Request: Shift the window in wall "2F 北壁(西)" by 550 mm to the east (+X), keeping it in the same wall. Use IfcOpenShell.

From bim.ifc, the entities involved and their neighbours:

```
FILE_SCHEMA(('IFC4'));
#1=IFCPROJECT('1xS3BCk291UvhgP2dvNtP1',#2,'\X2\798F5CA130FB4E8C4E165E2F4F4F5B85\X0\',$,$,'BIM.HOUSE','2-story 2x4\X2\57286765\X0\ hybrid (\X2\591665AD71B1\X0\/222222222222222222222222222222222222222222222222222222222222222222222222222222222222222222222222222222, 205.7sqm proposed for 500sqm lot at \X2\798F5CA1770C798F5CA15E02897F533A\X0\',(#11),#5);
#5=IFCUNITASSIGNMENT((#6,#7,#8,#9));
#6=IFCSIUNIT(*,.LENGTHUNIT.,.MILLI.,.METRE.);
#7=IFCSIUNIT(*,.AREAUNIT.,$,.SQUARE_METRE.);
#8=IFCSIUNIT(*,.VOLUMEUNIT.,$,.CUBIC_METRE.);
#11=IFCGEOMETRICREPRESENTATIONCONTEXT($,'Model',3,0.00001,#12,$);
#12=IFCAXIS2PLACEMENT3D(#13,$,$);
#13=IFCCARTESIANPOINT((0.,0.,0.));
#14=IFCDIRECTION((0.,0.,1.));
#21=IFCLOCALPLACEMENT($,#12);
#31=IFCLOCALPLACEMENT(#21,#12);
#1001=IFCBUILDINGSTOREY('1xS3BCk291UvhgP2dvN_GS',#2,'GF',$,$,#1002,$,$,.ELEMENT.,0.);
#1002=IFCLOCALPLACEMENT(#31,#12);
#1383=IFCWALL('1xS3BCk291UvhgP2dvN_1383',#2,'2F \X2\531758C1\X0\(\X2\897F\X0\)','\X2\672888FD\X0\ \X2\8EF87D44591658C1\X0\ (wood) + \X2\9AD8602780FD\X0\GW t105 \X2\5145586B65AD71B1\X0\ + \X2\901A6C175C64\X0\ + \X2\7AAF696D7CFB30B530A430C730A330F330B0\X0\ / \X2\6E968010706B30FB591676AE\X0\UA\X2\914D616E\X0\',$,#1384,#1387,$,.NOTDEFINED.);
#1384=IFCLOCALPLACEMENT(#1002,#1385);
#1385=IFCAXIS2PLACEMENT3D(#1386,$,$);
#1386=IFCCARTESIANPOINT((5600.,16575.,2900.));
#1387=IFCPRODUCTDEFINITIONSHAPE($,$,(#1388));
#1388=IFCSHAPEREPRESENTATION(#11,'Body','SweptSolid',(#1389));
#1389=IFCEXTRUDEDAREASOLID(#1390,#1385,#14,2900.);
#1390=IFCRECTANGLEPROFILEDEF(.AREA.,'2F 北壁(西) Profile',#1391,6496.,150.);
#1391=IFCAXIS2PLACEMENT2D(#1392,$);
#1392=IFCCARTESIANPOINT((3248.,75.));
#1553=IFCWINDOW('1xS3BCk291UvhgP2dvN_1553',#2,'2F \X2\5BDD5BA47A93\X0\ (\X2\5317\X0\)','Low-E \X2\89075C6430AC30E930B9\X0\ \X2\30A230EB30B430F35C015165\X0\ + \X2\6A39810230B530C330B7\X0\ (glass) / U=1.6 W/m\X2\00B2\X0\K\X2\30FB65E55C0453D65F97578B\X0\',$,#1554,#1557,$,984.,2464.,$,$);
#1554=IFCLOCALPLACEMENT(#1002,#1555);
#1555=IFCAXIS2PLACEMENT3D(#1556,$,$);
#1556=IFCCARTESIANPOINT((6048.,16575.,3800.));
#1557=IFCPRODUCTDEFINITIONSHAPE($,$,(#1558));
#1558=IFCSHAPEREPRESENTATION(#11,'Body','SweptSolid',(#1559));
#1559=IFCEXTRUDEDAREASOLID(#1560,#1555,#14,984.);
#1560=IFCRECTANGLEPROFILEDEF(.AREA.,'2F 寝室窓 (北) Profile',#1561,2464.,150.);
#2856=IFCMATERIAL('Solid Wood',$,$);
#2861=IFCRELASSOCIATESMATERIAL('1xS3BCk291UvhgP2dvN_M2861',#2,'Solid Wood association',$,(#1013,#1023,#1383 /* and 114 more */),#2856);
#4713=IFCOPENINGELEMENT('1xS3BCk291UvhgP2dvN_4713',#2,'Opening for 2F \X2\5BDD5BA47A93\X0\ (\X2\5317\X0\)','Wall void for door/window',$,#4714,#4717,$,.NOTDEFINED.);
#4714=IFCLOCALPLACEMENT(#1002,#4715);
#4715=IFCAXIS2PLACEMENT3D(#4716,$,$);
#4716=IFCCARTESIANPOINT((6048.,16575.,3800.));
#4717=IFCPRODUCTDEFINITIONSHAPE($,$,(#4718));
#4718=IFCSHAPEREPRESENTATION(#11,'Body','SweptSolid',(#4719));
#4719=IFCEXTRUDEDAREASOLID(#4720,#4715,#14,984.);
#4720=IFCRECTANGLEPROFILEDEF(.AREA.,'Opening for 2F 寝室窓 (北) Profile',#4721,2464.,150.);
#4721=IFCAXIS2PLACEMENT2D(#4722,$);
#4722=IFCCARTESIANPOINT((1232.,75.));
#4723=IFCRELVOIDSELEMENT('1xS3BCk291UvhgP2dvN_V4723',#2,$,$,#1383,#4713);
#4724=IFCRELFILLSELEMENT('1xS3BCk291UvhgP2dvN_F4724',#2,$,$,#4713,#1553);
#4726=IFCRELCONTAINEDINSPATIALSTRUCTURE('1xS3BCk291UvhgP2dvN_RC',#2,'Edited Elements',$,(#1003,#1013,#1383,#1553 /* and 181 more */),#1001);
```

```python
import ifcopenshell
import ifcopenshell.api.geometry
import ifcopenshell.util.placement

model = ifcopenshell.open("bim.ifc")

window = model.by_id(1553)
opening = window.FillsVoids[0].RelatingOpeningElement
wall = opening.VoidsElements[0].RelatingBuildingElement

wall_matrix = ifcopenshell.util.placement.get_local_placement(wall.ObjectPlacement)
shift = wall_matrix[:3, 0] * 550.0
before = ifcopenshell.util.placement.get_local_placement(window.ObjectPlacement)[:3, 3].copy()

# The window is not placed relative to its opening, so move both.
for product in (opening, window):
    matrix = ifcopenshell.util.placement.get_local_placement(product.ObjectPlacement)
    matrix[:3, 3] += shift
    ifcopenshell.api.geometry.edit_object_placement(model, product=product, matrix=matrix, is_si=False)

after = ifcopenshell.util.placement.get_local_placement(window.ObjectPlacement)[:3, 3]
print("window moved by", (after - before).round(3) + 0.0)

model.write("bim_updated.ifc")
```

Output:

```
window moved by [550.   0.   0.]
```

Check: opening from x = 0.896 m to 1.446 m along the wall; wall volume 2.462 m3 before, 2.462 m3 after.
